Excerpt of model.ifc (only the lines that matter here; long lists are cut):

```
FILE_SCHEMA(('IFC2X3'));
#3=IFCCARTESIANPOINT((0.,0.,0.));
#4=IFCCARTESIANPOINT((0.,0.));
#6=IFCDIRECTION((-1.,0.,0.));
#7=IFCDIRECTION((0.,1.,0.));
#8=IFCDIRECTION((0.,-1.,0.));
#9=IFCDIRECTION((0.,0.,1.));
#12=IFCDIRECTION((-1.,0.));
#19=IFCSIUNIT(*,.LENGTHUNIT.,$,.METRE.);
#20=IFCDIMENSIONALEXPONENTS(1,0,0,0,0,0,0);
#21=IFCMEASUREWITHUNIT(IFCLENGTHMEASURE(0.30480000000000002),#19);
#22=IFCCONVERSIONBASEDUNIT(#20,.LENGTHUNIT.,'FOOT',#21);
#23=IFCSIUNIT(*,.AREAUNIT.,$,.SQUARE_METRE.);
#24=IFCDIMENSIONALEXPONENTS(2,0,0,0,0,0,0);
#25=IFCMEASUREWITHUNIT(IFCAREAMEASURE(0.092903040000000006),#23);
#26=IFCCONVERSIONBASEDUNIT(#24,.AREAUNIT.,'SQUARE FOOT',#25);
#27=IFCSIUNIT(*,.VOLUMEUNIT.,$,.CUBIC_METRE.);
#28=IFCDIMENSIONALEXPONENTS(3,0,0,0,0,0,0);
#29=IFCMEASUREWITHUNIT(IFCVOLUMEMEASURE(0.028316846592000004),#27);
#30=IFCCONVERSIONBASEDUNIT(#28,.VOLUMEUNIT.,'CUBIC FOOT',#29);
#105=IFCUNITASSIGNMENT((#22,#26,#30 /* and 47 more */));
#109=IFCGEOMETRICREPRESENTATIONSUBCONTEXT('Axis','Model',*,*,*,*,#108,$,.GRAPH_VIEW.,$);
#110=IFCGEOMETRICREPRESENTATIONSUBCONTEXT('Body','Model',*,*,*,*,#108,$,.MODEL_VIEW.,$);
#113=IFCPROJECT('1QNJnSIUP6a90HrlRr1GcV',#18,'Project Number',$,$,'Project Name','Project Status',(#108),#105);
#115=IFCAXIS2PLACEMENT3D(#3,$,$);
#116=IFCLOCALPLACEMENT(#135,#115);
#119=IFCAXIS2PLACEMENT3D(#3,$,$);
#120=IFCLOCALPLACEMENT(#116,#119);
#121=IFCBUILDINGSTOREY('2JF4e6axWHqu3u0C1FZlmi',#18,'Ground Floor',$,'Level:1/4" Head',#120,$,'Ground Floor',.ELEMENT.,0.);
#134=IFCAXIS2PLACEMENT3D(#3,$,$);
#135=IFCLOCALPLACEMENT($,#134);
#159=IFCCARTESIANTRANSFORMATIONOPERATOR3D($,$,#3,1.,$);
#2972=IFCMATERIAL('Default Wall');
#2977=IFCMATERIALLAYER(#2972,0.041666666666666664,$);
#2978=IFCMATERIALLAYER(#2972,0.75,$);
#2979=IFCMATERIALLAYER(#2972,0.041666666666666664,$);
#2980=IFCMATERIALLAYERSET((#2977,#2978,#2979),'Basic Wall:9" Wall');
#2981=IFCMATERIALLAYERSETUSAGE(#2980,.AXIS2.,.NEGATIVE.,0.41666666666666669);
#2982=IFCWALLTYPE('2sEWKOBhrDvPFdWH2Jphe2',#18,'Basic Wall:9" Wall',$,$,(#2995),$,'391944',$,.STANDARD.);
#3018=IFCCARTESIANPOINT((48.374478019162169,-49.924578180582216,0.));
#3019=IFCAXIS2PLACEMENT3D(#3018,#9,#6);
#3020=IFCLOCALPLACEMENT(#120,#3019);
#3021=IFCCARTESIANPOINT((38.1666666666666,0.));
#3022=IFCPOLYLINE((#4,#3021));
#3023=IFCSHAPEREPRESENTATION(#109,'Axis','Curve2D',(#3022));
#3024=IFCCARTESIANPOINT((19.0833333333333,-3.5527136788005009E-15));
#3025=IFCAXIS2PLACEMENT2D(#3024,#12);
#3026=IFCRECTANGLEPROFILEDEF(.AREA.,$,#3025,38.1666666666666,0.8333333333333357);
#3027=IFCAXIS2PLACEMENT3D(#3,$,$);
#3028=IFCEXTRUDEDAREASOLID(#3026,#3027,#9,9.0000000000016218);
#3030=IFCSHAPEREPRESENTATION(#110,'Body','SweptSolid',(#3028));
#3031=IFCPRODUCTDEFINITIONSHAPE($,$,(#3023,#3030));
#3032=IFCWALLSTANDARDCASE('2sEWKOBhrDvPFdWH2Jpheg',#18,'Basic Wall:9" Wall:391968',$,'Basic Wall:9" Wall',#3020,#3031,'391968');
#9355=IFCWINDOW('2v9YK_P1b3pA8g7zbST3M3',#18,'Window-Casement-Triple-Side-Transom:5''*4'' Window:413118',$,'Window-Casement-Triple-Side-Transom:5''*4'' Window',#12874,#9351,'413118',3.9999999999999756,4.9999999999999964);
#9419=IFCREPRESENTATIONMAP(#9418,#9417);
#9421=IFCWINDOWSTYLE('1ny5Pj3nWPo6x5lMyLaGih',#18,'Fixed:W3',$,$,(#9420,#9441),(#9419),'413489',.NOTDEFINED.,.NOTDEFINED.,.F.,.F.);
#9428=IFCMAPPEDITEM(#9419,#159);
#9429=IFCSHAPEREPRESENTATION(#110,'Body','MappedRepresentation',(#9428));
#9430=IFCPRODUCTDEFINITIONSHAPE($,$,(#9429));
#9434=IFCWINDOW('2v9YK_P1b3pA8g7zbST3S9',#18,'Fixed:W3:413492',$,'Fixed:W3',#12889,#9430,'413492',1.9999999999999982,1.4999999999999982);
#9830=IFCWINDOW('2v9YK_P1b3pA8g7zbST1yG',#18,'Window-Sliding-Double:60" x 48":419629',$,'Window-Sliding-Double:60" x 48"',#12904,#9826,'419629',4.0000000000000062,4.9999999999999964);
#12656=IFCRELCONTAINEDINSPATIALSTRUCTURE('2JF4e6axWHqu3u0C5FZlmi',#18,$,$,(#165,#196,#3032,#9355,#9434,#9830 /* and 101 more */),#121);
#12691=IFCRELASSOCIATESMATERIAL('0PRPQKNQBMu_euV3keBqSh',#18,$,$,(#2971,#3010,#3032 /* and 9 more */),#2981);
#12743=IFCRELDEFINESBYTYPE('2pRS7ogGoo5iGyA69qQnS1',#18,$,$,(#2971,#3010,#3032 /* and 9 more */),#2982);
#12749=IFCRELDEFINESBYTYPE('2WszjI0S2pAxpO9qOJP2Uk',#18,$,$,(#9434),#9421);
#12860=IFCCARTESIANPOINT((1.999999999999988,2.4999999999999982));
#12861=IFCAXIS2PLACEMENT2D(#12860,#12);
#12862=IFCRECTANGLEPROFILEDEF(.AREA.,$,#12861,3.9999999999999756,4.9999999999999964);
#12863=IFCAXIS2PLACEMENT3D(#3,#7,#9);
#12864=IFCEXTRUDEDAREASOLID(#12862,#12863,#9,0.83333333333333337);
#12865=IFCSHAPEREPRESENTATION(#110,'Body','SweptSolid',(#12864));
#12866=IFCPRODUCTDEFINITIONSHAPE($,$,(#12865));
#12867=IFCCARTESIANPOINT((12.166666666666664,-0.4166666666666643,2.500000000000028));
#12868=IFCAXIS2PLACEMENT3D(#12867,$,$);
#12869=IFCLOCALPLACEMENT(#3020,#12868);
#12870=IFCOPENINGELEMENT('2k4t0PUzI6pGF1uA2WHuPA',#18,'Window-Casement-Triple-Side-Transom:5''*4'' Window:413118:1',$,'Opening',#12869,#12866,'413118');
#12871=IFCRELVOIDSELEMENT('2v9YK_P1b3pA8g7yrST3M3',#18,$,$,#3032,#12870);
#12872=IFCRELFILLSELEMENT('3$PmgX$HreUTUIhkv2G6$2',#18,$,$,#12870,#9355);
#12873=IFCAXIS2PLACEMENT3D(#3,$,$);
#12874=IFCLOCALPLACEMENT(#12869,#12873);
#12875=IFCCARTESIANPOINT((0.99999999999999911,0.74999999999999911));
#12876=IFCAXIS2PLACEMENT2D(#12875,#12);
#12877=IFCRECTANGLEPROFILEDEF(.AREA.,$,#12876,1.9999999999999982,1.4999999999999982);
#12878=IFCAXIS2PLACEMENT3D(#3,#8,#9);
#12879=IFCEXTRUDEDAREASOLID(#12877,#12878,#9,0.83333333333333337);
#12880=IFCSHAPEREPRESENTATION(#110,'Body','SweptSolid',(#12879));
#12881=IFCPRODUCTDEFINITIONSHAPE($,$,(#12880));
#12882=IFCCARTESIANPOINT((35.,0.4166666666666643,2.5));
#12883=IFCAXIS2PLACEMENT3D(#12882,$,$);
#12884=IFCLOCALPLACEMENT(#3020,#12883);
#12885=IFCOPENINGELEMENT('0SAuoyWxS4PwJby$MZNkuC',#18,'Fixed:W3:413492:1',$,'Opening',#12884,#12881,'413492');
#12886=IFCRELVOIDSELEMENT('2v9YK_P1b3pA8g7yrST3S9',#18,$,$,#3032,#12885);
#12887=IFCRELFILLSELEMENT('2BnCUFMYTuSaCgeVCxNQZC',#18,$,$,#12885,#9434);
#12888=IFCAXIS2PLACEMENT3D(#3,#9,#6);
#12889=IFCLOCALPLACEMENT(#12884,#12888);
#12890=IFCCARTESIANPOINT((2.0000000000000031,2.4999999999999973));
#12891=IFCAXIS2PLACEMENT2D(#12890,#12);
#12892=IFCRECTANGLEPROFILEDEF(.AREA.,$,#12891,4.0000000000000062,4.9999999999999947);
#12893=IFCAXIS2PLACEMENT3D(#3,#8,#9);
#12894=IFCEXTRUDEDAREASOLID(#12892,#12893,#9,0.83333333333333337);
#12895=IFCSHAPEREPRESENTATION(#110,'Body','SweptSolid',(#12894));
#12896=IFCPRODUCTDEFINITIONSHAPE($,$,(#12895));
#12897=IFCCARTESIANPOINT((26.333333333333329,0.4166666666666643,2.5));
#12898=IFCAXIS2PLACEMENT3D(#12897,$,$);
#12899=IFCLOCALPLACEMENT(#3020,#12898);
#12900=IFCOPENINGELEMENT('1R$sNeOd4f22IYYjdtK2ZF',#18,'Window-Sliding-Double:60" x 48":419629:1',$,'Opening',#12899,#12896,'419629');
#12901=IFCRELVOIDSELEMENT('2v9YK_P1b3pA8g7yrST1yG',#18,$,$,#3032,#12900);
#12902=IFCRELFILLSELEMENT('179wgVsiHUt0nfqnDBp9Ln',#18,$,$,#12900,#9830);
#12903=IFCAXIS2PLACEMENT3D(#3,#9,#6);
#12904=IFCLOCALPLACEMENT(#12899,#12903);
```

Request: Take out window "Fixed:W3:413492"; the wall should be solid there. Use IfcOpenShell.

```python
import ifcopenshell
import ifcopenshell.api.feature
import ifcopenshell.api.root
import ifcopenshell.geom
import ifcopenshell.util.shape

model = ifcopenshell.open("model.ifc")
settings = ifcopenshell.geom.settings()


def volume(element):
    """Net volume in cubic metres, openings subtracted."""
    shape = ifcopenshell.geom.create_shape(settings, element)
    return ifcopenshell.util.shape.get_volume(shape.geometry)


window = model.by_guid("2v9YK_P1b3pA8g7zbST3S9")
opening = window.FillsVoids[0].RelatingOpeningElement
wall = opening.VoidsElements[0].RelatingBuildingElement
before = volume(wall)

ifcopenshell.api.root.remove_product(model, product=window)
ifcopenshell.api.feature.remove_feature(model, feature=opening)

after = volume(wall)

print(f"wall volume {before:.3f} -> {after:.3f} m3")

model.write("model-out.ifc")
```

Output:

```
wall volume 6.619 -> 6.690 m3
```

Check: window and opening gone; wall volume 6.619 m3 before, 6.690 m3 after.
